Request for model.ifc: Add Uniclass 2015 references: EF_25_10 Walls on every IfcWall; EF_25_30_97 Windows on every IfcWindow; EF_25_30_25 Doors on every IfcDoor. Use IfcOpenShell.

First a look at what the model holds.

```python
import ifcopenshell

model = ifcopenshell.open("model.ifc")
print(model.schema)
print("classifications:", [c.Name for c in model.by_type("IfcClassification")])
for ifc_class in ("IfcDoor", "IfcRoof", "IfcStair", "IfcWall", "IfcWindow"):
    print(ifc_class, len(model.by_type(ifc_class)))
```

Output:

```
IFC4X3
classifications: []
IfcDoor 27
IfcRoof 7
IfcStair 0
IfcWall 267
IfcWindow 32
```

```python
import ifcopenshell
import ifcopenshell.api.classification

model = ifcopenshell.open("model.ifc")

system = ifcopenshell.api.classification.add_classification(model, classification="Uniclass 2015")

codes = {
    "IfcWall": ("EF_25_10", "Walls"),
    "IfcWindow": ("EF_25_30_97", "Windows"),
    "IfcDoor": ("EF_25_30_25", "Doors"),
}
for ifc_class, (code, name) in codes.items():
    products = model.by_type(ifc_class)
    ifcopenshell.api.classification.add_reference(
        model, products=products, classification=system, identification=code, name=name
    )
    print(code, len(products))

model.write("model-out.ifc")
```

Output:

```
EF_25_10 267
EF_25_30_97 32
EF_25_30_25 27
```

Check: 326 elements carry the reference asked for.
